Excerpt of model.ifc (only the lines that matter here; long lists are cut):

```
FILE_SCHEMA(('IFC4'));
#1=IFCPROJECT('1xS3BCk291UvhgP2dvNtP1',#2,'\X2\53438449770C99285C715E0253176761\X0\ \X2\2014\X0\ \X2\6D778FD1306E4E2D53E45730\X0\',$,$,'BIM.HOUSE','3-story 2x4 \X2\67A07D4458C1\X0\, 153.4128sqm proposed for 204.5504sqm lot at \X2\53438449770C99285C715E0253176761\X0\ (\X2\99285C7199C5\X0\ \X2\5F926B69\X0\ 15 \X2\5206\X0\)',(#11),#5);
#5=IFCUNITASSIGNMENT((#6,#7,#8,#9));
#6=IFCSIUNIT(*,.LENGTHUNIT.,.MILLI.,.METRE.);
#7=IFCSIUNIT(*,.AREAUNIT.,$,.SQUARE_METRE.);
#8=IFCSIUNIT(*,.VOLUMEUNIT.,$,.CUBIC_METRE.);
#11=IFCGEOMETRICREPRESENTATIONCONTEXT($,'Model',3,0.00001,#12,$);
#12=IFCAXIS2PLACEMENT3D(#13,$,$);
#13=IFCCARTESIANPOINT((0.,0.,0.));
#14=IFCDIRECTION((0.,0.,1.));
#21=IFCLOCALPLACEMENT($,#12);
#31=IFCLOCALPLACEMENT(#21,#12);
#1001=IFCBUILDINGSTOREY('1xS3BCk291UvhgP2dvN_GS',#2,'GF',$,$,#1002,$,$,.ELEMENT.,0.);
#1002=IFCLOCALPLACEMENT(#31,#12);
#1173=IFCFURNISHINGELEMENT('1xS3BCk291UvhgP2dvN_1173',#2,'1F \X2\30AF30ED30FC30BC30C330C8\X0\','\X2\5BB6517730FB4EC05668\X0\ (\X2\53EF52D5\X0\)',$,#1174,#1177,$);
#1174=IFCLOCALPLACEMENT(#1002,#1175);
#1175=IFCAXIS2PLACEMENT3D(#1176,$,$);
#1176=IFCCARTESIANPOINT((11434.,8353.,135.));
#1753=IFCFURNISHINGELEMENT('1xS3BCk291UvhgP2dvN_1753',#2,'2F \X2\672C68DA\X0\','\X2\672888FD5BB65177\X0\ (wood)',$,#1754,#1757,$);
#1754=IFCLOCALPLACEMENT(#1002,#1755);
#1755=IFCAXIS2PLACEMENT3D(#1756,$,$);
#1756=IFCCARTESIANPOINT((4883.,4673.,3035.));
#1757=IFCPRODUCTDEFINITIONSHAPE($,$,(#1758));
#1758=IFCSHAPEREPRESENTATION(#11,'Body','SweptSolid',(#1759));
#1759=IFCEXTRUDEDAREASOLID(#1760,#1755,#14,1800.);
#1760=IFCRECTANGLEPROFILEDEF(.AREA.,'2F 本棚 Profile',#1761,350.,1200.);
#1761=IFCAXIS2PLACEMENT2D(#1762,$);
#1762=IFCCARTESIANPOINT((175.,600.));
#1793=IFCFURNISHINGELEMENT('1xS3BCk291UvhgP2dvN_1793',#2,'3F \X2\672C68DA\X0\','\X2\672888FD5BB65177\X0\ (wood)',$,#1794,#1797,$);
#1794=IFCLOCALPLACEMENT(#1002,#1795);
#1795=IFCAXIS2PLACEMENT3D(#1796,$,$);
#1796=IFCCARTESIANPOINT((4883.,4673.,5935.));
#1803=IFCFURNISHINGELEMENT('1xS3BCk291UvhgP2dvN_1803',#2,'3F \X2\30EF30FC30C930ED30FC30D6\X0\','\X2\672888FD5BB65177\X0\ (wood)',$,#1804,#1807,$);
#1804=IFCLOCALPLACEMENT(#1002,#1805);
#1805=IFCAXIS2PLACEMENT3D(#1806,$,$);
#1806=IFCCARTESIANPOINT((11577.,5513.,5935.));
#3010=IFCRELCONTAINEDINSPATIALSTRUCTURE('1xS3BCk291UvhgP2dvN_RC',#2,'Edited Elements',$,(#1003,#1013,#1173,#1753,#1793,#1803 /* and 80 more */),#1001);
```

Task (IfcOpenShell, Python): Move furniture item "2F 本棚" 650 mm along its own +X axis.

```python
import ifcopenshell
import ifcopenshell.api.geometry
import ifcopenshell.util.placement
import ifcopenshell.util.unit

model = ifcopenshell.open("model.ifc")
unit_scale = ifcopenshell.util.unit.calculate_unit_scale(model)

item = model.by_id(1753)
matrix = ifcopenshell.util.placement.get_local_placement(item.ObjectPlacement)
matrix[:3, 3] += matrix[:3, 0] * 0.65 / unit_scale
ifcopenshell.api.geometry.edit_object_placement(model, product=item, matrix=matrix, is_si=False)

print(ifcopenshell.util.placement.get_local_placement(item.ObjectPlacement).round(3) + 0.0)

model.write("model_edited.ifc")
```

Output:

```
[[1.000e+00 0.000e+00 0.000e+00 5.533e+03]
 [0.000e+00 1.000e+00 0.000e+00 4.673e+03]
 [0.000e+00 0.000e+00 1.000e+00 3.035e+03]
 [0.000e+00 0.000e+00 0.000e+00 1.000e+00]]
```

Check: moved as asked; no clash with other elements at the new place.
